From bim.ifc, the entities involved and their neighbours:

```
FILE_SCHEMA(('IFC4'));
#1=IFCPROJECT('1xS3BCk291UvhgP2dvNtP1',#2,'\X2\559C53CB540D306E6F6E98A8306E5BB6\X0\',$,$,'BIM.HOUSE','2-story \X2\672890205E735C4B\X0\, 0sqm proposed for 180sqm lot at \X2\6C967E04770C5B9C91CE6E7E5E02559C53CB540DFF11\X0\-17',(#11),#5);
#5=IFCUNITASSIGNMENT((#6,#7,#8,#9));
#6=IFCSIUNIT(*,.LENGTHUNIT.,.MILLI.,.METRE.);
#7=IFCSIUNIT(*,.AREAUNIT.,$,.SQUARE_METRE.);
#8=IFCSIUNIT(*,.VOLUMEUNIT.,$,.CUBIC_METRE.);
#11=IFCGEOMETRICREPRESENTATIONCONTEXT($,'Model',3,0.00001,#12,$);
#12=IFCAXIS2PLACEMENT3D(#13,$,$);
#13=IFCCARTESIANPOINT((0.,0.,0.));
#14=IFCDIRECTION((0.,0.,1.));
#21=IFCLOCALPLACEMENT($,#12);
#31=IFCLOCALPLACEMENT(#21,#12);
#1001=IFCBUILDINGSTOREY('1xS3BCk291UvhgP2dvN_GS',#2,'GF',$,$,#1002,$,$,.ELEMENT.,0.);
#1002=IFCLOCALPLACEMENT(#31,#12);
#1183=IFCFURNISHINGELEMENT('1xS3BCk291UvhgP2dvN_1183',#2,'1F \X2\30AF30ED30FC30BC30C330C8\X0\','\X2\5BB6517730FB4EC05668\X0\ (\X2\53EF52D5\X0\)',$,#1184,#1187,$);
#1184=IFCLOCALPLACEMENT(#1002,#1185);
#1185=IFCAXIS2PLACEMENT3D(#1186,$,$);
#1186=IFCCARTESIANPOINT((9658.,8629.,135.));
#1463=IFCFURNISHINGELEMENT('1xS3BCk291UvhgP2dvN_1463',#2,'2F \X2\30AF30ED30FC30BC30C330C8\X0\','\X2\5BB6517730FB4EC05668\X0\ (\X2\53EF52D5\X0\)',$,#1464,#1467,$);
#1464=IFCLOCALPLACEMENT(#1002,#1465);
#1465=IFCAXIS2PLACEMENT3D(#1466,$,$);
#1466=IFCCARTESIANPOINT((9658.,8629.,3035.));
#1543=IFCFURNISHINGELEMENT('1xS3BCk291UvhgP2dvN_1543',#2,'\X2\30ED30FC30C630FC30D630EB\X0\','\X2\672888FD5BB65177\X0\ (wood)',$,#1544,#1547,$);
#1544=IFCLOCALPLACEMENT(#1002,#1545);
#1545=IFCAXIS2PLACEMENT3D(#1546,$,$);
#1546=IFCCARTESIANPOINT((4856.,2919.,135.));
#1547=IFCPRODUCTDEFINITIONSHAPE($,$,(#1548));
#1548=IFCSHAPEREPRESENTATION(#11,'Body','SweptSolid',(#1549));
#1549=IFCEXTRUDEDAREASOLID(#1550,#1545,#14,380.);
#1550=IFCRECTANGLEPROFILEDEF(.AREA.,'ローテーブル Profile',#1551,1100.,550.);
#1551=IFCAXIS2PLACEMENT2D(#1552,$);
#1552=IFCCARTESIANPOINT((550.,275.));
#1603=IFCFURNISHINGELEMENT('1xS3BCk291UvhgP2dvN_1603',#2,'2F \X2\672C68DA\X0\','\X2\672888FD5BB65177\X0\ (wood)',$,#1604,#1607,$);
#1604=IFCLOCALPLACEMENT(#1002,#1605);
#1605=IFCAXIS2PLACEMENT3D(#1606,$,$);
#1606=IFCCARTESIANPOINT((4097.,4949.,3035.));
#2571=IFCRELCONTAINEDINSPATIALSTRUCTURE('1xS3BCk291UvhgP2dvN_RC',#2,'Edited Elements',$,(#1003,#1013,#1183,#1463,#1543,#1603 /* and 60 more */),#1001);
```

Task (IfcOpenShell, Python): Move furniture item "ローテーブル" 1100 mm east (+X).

```python
import ifcopenshell
import ifcopenshell.api.geometry
import ifcopenshell.util.placement
import ifcopenshell.util.unit

model = ifcopenshell.open("bim.ifc")
unit_scale = ifcopenshell.util.unit.calculate_unit_scale(model)

item = model.by_id(1543)
matrix = ifcopenshell.util.placement.get_local_placement(item.ObjectPlacement)
matrix[0, 3] += 1.1 / unit_scale
ifcopenshell.api.geometry.edit_object_placement(model, product=item, matrix=matrix, is_si=False)

print(ifcopenshell.util.placement.get_local_placement(item.ObjectPlacement).round(3) + 0.0)

model.write("bim-out.ifc")
```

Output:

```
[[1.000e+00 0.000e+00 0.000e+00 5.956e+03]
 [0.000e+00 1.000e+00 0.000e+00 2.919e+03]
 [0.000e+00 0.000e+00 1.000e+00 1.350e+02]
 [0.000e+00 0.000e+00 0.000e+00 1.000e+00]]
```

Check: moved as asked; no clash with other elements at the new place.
